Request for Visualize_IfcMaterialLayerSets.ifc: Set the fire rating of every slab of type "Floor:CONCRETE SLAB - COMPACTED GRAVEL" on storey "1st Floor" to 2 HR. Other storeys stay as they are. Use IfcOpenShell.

First a look at what the model holds.

```python
import ifcopenshell
import ifcopenshell.util.element

model = ifcopenshell.open("Visualize_IfcMaterialLayerSets.ifc")
print(model.schema)
storey = next(s for s in model.by_type("IfcBuildingStorey") if s.Name == "1st Floor")
slabs = [e for e in ifcopenshell.util.element.get_decomposition(storey) if e.is_a("IfcSlab")]
seen = {}
for e in slabs:
    element_type = ifcopenshell.util.element.get_type(e)
    key = (element_type.Name if element_type != e and element_type else None, ifcopenshell.util.element.get_pset(e, "Pset_SlabCommon", "FireRating"))
    seen[key] = seen.get(key, 0) + 1
for (name, value), count in sorted(seen.items(), key=str):
    print(count, "x", name, "|", value)
```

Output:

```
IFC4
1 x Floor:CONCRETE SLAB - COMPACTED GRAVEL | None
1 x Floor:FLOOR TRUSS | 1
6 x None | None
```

```python
import ifcopenshell
import ifcopenshell.api.pset
import ifcopenshell.util.element

model = ifcopenshell.open("Visualize_IfcMaterialLayerSets.ifc")

storey = next(s for s in model.by_type("IfcBuildingStorey") if s.Name == "1st Floor")
slabs = [e for e in ifcopenshell.util.element.get_decomposition(storey) if e.is_a("IfcSlab")]

count = 0
for e in slabs:
    element_type = ifcopenshell.util.element.get_type(e)
    if element_type in (None, e) or element_type.Name != "Floor:CONCRETE SLAB - COMPACTED GRAVEL":
        continue
    # add_pset returns the element's existing set when there is one.
    pset = ifcopenshell.api.pset.add_pset(model, product=e, name="Pset_SlabCommon")
    ifcopenshell.api.pset.edit_pset(model, pset=pset, properties={"FireRating": "2 HR"})
    count += 1

print(count, "slabs updated")

model.write("Visualize_IfcMaterialLayerSets-out.ifc")
```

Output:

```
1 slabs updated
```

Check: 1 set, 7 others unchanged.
